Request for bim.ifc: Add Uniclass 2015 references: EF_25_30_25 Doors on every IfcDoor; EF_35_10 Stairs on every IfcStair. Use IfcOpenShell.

First a look at what the model holds.

```python
import ifcopenshell

model = ifcopenshell.open("bim.ifc")
print(model.schema)
print("classifications:", [c.Name for c in model.by_type("IfcClassification")])
for ifc_class in ("IfcDoor", "IfcRoof", "IfcStair", "IfcWall", "IfcWindow"):
    print(ifc_class, len(model.by_type(ifc_class)))
```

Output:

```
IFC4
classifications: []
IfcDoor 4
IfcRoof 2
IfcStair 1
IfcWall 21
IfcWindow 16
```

```python
import ifcopenshell
import ifcopenshell.api.classification

model = ifcopenshell.open("bim.ifc")

system = ifcopenshell.api.classification.add_classification(model, classification="Uniclass 2015")

codes = {
    "IfcDoor": ("EF_25_30_25", "Doors"),
    "IfcStair": ("EF_35_10", "Stairs"),
}
for ifc_class, (code, name) in codes.items():
    products = model.by_type(ifc_class)
    ifcopenshell.api.classification.add_reference(
        model, products=products, classification=system, identification=code, name=name
    )
    print(code, len(products))

model.write("bim_v2.ifc")
```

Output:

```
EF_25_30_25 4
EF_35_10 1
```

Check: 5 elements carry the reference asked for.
